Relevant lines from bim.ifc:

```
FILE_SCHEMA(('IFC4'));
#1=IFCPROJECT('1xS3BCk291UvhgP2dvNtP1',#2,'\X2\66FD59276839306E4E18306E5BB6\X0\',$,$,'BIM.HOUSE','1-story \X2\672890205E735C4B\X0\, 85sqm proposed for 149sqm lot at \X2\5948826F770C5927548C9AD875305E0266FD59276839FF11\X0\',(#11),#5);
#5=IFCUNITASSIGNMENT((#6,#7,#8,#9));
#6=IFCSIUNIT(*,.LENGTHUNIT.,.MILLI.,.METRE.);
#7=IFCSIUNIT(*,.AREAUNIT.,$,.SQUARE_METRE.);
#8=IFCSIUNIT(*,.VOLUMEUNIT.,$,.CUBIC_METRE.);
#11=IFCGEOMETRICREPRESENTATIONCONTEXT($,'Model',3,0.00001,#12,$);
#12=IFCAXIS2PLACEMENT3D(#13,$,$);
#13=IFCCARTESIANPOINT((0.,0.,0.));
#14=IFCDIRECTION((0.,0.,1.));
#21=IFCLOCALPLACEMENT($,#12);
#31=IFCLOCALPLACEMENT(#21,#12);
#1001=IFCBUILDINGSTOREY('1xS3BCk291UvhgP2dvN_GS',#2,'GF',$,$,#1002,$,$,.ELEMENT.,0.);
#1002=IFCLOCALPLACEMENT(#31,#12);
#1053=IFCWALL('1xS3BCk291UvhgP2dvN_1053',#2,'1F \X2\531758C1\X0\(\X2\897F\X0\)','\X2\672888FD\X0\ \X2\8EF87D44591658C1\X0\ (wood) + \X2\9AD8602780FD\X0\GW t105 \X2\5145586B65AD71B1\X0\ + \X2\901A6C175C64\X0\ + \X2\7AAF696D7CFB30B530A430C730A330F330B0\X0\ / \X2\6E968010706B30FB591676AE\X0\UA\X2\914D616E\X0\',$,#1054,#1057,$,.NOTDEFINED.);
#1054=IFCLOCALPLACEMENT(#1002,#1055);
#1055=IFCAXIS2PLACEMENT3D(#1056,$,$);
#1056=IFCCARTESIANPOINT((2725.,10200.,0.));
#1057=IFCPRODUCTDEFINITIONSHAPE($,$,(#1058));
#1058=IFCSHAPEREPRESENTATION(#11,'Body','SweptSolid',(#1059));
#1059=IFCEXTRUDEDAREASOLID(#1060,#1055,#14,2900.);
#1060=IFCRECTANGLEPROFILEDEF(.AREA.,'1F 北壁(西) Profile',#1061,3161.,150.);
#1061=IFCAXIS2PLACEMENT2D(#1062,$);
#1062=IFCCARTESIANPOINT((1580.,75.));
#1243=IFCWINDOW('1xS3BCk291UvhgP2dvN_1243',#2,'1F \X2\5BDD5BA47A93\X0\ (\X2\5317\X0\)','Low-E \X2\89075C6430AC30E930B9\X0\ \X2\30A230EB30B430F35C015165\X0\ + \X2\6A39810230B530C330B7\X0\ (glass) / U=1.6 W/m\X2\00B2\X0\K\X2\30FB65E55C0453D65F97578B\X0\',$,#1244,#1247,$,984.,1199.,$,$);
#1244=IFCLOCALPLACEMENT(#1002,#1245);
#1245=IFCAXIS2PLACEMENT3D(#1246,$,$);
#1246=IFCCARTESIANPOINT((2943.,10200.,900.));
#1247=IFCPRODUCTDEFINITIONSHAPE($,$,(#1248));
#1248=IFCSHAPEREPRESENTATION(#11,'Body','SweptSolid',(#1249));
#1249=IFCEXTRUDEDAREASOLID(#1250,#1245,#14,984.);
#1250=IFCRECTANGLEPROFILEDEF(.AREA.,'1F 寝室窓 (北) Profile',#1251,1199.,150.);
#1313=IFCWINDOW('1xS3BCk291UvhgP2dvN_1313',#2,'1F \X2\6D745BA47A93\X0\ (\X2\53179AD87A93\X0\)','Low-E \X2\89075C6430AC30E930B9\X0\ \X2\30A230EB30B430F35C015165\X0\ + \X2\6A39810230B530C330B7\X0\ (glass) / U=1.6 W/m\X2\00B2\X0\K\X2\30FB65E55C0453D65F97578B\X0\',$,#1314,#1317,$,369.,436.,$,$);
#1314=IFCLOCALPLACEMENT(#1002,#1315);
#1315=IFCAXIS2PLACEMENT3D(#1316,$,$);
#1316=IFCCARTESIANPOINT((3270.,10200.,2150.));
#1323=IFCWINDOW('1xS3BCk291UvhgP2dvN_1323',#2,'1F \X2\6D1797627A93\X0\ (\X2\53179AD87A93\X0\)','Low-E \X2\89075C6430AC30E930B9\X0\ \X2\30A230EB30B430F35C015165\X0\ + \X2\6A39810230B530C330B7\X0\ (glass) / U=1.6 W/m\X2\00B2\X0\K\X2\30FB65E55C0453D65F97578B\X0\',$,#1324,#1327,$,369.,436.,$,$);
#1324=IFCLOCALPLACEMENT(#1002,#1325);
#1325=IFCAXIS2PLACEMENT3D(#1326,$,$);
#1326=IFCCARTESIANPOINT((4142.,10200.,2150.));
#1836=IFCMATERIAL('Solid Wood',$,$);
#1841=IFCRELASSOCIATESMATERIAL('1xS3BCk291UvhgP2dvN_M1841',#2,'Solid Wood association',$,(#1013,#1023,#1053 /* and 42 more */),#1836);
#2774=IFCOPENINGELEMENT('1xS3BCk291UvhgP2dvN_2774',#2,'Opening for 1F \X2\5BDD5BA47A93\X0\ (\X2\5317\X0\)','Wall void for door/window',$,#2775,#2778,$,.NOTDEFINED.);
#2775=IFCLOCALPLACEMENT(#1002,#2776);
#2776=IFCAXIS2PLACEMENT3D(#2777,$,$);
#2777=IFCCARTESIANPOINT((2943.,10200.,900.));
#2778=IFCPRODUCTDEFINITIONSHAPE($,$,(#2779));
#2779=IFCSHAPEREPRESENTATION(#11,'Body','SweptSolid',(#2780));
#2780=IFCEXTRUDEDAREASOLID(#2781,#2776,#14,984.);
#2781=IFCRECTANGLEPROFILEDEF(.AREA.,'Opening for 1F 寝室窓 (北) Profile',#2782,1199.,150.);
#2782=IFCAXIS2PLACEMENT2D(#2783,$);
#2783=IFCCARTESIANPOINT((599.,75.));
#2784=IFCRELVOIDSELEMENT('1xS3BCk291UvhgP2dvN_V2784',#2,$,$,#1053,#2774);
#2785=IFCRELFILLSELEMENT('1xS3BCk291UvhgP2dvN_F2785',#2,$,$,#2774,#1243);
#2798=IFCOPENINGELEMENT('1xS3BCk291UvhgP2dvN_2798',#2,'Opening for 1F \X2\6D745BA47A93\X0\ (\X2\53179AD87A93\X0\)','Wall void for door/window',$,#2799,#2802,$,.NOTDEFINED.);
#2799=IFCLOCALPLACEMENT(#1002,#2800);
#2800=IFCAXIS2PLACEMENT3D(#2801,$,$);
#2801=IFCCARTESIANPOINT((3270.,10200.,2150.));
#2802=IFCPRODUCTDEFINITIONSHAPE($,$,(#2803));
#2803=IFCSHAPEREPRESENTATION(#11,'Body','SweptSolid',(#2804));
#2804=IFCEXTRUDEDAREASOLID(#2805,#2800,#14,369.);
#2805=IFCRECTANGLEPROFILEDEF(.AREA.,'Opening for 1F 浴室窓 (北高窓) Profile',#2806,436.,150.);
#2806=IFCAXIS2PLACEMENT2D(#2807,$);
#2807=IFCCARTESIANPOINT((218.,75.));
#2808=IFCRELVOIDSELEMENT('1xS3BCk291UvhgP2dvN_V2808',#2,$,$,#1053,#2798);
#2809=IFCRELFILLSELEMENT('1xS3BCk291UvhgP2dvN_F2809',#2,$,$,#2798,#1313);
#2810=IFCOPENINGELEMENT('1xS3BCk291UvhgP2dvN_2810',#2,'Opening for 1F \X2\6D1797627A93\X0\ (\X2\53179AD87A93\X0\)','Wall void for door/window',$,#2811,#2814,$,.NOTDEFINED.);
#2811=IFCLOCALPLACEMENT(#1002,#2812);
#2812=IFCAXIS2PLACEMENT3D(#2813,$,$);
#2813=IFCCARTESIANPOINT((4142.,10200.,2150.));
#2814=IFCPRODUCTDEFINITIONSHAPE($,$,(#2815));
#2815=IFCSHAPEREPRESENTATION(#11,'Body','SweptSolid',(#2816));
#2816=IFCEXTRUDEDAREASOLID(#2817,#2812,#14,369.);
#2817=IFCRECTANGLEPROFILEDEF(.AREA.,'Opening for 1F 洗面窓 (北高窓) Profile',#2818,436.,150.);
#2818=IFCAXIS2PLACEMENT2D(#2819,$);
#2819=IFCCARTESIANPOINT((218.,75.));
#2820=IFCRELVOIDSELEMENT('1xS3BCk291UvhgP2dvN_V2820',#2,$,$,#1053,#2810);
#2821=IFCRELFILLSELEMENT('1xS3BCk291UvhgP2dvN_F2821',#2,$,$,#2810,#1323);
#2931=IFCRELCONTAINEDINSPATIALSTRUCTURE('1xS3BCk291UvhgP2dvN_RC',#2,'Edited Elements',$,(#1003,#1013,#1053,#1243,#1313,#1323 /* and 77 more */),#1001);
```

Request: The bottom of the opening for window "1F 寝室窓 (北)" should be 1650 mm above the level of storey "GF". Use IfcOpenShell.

```python
import numpy as np
import ifcopenshell
import ifcopenshell.api.geometry
import ifcopenshell.geom
import ifcopenshell.util.element
import ifcopenshell.util.placement
import ifcopenshell.util.shape
import ifcopenshell.util.unit

model = ifcopenshell.open("bim.ifc")
unit_scale = ifcopenshell.util.unit.calculate_unit_scale(model)

window = model.by_guid("1xS3BCk291UvhgP2dvN_1243")
opening = window.FillsVoids[0].RelatingOpeningElement
storey = ifcopenshell.util.element.get_container(window, ifc_class="IfcBuildingStorey")
level = ifcopenshell.util.placement.get_local_placement(storey.ObjectPlacement)[2, 3]

# The opening's origin need not be at the sill, so measure its lowest point.
shape = ifcopenshell.geom.create_shape(ifcopenshell.geom.settings(), opening)
bottom = ifcopenshell.util.shape.get_shape_bottom_elevation(shape, shape.geometry) / unit_scale
dz = level + 1.65 / unit_scale - bottom

shift = np.array([0.0, 0.0, dz])
# The window is not placed relative to its opening, so move both.
for product in (opening, window):
    matrix = ifcopenshell.util.placement.get_local_placement(product.ObjectPlacement)
    matrix[:3, 3] += shift
    ifcopenshell.api.geometry.edit_object_placement(model, product=product, matrix=matrix, is_si=False)

print(f"moved by {dz * unit_scale:+.3f} m")

model.write("bim_edited.ifc")
```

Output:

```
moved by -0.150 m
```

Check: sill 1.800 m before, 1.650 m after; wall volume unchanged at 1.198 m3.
